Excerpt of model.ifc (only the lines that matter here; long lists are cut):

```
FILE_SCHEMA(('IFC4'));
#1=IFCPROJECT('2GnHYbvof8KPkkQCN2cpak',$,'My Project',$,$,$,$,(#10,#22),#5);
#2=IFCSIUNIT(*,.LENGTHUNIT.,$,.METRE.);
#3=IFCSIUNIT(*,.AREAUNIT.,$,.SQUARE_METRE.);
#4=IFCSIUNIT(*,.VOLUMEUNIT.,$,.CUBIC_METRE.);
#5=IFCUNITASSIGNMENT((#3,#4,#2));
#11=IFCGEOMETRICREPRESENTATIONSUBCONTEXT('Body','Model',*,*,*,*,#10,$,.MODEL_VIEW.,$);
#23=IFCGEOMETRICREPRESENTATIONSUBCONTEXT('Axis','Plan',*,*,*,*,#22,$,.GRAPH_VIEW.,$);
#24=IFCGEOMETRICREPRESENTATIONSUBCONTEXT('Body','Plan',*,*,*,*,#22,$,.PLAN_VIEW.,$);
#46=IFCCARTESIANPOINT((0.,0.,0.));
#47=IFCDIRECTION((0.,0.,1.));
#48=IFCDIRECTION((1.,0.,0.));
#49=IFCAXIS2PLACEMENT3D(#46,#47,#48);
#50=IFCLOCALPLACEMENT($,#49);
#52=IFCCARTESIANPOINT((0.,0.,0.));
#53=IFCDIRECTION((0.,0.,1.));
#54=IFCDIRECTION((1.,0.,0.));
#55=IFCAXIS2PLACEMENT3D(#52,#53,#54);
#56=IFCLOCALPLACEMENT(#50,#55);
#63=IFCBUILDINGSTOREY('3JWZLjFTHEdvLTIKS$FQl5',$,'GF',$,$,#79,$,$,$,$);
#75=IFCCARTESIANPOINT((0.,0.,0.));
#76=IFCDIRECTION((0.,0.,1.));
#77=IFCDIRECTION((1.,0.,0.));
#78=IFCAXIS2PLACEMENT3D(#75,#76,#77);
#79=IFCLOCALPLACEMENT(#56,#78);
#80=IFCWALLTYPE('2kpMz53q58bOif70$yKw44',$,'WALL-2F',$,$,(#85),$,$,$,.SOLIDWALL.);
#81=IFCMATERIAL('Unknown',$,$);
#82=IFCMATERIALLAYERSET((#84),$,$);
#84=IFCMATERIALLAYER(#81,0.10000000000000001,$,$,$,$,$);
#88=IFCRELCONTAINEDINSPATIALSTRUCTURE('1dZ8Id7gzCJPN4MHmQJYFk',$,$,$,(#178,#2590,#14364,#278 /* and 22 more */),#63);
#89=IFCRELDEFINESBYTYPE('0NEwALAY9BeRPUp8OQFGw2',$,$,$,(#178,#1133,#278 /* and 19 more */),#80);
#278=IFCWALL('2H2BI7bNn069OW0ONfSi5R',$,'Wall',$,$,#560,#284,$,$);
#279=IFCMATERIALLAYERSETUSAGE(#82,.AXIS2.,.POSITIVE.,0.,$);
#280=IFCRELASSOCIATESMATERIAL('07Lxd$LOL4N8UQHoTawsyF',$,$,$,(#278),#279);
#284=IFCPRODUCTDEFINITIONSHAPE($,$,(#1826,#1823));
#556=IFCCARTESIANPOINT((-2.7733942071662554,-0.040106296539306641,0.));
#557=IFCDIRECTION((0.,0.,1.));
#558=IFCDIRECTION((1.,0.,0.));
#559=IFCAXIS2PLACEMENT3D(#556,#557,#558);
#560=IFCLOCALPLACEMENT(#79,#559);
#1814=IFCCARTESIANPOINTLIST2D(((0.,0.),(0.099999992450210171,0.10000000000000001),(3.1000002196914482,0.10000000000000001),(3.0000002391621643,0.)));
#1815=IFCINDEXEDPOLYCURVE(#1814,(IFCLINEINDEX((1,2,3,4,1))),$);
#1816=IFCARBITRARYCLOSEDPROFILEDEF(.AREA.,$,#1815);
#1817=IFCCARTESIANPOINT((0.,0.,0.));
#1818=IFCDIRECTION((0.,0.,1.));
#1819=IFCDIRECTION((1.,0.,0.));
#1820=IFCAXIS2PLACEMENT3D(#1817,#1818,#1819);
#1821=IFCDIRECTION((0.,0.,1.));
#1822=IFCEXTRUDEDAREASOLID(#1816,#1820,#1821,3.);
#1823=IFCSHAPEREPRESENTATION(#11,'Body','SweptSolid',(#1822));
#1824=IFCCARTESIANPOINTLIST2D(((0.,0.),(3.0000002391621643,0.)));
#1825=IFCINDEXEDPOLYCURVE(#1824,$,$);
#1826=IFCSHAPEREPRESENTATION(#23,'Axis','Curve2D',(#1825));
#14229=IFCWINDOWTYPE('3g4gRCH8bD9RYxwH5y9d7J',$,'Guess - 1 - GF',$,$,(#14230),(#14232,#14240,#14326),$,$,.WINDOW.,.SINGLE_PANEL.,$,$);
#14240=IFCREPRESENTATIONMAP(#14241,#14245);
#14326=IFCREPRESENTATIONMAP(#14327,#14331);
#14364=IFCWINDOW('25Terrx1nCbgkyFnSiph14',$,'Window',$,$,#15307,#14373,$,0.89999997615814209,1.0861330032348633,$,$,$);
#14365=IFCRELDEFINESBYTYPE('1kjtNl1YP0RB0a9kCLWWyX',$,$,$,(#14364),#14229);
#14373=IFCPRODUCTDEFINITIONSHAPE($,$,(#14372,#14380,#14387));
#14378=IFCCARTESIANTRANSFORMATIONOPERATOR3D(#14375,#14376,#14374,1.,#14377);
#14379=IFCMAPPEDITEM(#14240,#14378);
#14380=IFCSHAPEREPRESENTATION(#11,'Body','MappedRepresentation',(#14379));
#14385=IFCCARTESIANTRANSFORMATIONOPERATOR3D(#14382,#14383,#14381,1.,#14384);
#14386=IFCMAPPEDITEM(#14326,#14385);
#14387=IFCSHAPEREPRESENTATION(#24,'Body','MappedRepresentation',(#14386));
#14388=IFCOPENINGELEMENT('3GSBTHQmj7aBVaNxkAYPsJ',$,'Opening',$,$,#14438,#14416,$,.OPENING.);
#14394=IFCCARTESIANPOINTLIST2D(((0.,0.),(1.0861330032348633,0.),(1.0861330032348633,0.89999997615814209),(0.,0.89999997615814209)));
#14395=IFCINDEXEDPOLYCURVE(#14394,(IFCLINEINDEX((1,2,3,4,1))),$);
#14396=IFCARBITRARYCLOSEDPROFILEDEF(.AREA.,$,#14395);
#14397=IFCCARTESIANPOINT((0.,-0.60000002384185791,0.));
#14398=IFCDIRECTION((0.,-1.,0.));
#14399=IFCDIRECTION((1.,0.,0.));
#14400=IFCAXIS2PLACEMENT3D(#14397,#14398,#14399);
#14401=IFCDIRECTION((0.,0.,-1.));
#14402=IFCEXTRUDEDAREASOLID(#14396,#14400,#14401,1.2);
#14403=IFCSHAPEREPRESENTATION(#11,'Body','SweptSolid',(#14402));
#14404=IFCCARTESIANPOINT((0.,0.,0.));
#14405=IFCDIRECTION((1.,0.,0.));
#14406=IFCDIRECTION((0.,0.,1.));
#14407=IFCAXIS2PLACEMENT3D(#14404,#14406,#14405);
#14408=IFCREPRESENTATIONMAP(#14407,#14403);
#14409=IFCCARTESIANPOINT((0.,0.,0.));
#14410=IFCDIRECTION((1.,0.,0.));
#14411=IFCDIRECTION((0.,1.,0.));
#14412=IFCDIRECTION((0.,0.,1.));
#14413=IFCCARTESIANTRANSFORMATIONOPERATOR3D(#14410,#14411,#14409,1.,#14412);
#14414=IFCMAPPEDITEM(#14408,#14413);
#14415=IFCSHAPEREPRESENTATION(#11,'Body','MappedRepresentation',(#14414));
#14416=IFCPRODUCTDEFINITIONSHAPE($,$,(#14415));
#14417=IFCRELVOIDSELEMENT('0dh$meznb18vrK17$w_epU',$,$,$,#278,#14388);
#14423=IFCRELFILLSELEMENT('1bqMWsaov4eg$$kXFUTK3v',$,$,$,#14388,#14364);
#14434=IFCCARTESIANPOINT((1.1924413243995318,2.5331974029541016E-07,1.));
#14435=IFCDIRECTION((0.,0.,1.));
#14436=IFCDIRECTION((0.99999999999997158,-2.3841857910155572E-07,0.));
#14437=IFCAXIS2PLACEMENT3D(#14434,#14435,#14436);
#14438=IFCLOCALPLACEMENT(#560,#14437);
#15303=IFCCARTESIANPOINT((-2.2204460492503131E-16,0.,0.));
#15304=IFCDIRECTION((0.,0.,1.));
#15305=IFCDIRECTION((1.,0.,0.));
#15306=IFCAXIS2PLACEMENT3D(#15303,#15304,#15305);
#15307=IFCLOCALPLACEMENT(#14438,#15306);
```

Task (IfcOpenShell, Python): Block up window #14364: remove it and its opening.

```python
import ifcopenshell
import ifcopenshell.api.feature
import ifcopenshell.api.root
import ifcopenshell.geom
import ifcopenshell.util.shape

model = ifcopenshell.open("model.ifc")
settings = ifcopenshell.geom.settings()


def volume(element):
    """Net volume in cubic metres, openings subtracted."""
    shape = ifcopenshell.geom.create_shape(settings, element)
    return ifcopenshell.util.shape.get_volume(shape.geometry)


window = model.by_guid("25Terrx1nCbgkyFnSiph14")
opening = window.FillsVoids[0].RelatingOpeningElement
wall = opening.VoidsElements[0].RelatingBuildingElement
before = volume(wall)

ifcopenshell.api.root.remove_product(model, product=window)
ifcopenshell.api.feature.remove_feature(model, feature=opening)

after = volume(wall)

print(f"wall volume {before:.3f} -> {after:.3f} m3")

model.write("model_v2.ifc")
```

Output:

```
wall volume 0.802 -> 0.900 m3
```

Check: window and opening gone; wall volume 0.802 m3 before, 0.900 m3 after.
